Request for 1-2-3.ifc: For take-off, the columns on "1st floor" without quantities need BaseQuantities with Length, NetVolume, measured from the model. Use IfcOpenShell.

First a look at what the model holds.

```python
import ifcopenshell
import ifcopenshell.util.element
import ifcopenshell.util.unit

model = ifcopenshell.open("1-2-3.ifc")
print(model.schema)
for unit_type in ("LENGTHUNIT", "AREAUNIT", "VOLUMEUNIT"):
    print(unit_type, ifcopenshell.util.unit.calculate_unit_scale(model, unit_type))
storey = next(s for s in model.by_type("IfcBuildingStorey") if s.Name == "1st floor")
columns = [e for e in ifcopenshell.util.element.get_decomposition(storey) if e.is_a("IfcColumn")]
for e in sorted(columns, key=lambda e: e.id()):
    print(e.id(), e.is_a(), e.Name, list(ifcopenshell.util.element.get_psets(e, qtos_only=True)), sep=" | ")
```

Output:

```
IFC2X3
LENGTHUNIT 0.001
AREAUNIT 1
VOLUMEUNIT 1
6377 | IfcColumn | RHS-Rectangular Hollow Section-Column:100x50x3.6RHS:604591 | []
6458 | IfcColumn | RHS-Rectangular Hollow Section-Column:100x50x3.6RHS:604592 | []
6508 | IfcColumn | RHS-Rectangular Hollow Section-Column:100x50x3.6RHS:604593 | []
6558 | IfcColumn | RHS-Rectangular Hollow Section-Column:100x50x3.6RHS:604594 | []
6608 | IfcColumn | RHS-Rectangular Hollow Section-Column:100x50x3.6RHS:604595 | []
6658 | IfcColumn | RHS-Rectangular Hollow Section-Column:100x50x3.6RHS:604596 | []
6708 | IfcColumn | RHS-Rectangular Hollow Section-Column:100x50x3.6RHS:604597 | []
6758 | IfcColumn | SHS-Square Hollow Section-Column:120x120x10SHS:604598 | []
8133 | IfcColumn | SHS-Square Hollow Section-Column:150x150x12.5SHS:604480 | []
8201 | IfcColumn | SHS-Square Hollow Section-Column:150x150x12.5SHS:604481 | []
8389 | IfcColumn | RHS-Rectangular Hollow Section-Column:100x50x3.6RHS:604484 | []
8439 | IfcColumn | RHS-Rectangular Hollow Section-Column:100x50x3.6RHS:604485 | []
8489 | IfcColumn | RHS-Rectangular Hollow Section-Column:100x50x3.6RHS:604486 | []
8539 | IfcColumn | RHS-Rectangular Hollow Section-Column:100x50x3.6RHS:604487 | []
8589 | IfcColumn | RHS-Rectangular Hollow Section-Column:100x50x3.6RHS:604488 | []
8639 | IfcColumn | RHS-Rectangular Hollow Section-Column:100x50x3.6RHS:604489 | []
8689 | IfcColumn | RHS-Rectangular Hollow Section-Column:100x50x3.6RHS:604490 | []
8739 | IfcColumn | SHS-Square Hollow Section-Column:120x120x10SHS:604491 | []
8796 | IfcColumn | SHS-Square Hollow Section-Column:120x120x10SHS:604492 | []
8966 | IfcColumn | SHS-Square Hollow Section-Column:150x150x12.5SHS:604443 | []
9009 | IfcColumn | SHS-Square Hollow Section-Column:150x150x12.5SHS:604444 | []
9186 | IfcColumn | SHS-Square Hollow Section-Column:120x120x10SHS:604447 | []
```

```python
import ifcopenshell
import ifcopenshell.api.pset
import ifcopenshell.geom
import ifcopenshell.util.element
import ifcopenshell.util.shape
import ifcopenshell.util.unit

model = ifcopenshell.open("1-2-3.ifc")
unit_scale = ifcopenshell.util.unit.calculate_unit_scale(model)
volume_scale = ifcopenshell.util.unit.calculate_unit_scale(model, "VOLUMEUNIT")
settings = ifcopenshell.geom.settings()

storey = next(s for s in model.by_type("IfcBuildingStorey") if s.Name == "1st floor")
columns = [e for e in ifcopenshell.util.element.get_decomposition(storey) if e.is_a("IfcColumn")]

for e in sorted(columns, key=lambda e: e.id()):
    if ifcopenshell.util.element.get_psets(e, qtos_only=True, should_inherit=False):
        continue
    # Geometry comes back in metres, in the element's own axes.
    shape = ifcopenshell.geom.create_shape(settings, e)
    values = {
        "Length": ifcopenshell.util.shape.get_z(shape.geometry) / unit_scale,
        "NetVolume": ifcopenshell.util.shape.get_volume(shape.geometry) / volume_scale,
    }
    qto = ifcopenshell.api.pset.add_qto(model, product=e, name="BaseQuantities")
    ifcopenshell.api.pset.edit_qto(model, qto=qto, properties=values)
    print(e.id(), {k: round(v, 3) for k, v in values.items()})

model.write("1-2-3-out.ifc")
```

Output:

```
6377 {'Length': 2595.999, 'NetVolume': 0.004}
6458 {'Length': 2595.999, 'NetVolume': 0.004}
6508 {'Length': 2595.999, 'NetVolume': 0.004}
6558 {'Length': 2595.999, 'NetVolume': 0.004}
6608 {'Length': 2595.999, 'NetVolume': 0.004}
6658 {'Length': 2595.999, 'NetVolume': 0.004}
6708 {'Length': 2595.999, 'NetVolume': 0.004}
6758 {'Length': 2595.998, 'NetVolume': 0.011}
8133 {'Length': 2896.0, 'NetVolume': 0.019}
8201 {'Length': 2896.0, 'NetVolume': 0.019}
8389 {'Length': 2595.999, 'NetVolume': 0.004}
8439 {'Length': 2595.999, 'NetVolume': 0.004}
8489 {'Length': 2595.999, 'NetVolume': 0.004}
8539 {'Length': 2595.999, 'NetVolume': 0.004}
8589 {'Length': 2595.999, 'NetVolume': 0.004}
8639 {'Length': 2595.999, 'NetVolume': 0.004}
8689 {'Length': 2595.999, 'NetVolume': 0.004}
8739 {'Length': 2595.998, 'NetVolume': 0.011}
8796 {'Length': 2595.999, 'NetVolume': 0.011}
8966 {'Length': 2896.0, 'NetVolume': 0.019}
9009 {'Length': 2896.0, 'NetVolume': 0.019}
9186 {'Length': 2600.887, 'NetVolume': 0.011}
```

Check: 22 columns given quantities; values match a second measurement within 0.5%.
